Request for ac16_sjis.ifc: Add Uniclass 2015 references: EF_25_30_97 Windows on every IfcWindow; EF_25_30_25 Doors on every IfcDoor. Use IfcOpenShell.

First a look at what the model holds.

```python
import ifcopenshell

model = ifcopenshell.open("ac16_sjis.ifc")
print(model.schema)
print("classifications:", [c.Name for c in model.by_type("IfcClassification")])
for ifc_class in ("IfcDoor", "IfcRoof", "IfcStair", "IfcWall", "IfcWindow"):
    print(ifc_class, len(model.by_type(ifc_class)))
```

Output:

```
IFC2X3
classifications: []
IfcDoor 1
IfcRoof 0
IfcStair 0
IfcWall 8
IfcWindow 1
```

```python
import ifcopenshell
import ifcopenshell.api.classification

model = ifcopenshell.open("ac16_sjis.ifc")

# IFC2X3 requires Source and Edition and has no link from the project to the system.
system = model.create_entity("IfcClassification", Source="NBS", Edition="2015", Name="Uniclass 2015")

codes = {
    "IfcWindow": ("EF_25_30_97", "Windows"),
    "IfcDoor": ("EF_25_30_25", "Doors"),
}
for ifc_class, (code, name) in codes.items():
    products = model.by_type(ifc_class)
    ifcopenshell.api.classification.add_reference(
        model, products=products, classification=system, identification=code, name=name
    )
    print(code, len(products))

model.write("ac16_sjis_v2.ifc")
```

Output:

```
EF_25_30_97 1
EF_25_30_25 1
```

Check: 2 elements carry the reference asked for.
